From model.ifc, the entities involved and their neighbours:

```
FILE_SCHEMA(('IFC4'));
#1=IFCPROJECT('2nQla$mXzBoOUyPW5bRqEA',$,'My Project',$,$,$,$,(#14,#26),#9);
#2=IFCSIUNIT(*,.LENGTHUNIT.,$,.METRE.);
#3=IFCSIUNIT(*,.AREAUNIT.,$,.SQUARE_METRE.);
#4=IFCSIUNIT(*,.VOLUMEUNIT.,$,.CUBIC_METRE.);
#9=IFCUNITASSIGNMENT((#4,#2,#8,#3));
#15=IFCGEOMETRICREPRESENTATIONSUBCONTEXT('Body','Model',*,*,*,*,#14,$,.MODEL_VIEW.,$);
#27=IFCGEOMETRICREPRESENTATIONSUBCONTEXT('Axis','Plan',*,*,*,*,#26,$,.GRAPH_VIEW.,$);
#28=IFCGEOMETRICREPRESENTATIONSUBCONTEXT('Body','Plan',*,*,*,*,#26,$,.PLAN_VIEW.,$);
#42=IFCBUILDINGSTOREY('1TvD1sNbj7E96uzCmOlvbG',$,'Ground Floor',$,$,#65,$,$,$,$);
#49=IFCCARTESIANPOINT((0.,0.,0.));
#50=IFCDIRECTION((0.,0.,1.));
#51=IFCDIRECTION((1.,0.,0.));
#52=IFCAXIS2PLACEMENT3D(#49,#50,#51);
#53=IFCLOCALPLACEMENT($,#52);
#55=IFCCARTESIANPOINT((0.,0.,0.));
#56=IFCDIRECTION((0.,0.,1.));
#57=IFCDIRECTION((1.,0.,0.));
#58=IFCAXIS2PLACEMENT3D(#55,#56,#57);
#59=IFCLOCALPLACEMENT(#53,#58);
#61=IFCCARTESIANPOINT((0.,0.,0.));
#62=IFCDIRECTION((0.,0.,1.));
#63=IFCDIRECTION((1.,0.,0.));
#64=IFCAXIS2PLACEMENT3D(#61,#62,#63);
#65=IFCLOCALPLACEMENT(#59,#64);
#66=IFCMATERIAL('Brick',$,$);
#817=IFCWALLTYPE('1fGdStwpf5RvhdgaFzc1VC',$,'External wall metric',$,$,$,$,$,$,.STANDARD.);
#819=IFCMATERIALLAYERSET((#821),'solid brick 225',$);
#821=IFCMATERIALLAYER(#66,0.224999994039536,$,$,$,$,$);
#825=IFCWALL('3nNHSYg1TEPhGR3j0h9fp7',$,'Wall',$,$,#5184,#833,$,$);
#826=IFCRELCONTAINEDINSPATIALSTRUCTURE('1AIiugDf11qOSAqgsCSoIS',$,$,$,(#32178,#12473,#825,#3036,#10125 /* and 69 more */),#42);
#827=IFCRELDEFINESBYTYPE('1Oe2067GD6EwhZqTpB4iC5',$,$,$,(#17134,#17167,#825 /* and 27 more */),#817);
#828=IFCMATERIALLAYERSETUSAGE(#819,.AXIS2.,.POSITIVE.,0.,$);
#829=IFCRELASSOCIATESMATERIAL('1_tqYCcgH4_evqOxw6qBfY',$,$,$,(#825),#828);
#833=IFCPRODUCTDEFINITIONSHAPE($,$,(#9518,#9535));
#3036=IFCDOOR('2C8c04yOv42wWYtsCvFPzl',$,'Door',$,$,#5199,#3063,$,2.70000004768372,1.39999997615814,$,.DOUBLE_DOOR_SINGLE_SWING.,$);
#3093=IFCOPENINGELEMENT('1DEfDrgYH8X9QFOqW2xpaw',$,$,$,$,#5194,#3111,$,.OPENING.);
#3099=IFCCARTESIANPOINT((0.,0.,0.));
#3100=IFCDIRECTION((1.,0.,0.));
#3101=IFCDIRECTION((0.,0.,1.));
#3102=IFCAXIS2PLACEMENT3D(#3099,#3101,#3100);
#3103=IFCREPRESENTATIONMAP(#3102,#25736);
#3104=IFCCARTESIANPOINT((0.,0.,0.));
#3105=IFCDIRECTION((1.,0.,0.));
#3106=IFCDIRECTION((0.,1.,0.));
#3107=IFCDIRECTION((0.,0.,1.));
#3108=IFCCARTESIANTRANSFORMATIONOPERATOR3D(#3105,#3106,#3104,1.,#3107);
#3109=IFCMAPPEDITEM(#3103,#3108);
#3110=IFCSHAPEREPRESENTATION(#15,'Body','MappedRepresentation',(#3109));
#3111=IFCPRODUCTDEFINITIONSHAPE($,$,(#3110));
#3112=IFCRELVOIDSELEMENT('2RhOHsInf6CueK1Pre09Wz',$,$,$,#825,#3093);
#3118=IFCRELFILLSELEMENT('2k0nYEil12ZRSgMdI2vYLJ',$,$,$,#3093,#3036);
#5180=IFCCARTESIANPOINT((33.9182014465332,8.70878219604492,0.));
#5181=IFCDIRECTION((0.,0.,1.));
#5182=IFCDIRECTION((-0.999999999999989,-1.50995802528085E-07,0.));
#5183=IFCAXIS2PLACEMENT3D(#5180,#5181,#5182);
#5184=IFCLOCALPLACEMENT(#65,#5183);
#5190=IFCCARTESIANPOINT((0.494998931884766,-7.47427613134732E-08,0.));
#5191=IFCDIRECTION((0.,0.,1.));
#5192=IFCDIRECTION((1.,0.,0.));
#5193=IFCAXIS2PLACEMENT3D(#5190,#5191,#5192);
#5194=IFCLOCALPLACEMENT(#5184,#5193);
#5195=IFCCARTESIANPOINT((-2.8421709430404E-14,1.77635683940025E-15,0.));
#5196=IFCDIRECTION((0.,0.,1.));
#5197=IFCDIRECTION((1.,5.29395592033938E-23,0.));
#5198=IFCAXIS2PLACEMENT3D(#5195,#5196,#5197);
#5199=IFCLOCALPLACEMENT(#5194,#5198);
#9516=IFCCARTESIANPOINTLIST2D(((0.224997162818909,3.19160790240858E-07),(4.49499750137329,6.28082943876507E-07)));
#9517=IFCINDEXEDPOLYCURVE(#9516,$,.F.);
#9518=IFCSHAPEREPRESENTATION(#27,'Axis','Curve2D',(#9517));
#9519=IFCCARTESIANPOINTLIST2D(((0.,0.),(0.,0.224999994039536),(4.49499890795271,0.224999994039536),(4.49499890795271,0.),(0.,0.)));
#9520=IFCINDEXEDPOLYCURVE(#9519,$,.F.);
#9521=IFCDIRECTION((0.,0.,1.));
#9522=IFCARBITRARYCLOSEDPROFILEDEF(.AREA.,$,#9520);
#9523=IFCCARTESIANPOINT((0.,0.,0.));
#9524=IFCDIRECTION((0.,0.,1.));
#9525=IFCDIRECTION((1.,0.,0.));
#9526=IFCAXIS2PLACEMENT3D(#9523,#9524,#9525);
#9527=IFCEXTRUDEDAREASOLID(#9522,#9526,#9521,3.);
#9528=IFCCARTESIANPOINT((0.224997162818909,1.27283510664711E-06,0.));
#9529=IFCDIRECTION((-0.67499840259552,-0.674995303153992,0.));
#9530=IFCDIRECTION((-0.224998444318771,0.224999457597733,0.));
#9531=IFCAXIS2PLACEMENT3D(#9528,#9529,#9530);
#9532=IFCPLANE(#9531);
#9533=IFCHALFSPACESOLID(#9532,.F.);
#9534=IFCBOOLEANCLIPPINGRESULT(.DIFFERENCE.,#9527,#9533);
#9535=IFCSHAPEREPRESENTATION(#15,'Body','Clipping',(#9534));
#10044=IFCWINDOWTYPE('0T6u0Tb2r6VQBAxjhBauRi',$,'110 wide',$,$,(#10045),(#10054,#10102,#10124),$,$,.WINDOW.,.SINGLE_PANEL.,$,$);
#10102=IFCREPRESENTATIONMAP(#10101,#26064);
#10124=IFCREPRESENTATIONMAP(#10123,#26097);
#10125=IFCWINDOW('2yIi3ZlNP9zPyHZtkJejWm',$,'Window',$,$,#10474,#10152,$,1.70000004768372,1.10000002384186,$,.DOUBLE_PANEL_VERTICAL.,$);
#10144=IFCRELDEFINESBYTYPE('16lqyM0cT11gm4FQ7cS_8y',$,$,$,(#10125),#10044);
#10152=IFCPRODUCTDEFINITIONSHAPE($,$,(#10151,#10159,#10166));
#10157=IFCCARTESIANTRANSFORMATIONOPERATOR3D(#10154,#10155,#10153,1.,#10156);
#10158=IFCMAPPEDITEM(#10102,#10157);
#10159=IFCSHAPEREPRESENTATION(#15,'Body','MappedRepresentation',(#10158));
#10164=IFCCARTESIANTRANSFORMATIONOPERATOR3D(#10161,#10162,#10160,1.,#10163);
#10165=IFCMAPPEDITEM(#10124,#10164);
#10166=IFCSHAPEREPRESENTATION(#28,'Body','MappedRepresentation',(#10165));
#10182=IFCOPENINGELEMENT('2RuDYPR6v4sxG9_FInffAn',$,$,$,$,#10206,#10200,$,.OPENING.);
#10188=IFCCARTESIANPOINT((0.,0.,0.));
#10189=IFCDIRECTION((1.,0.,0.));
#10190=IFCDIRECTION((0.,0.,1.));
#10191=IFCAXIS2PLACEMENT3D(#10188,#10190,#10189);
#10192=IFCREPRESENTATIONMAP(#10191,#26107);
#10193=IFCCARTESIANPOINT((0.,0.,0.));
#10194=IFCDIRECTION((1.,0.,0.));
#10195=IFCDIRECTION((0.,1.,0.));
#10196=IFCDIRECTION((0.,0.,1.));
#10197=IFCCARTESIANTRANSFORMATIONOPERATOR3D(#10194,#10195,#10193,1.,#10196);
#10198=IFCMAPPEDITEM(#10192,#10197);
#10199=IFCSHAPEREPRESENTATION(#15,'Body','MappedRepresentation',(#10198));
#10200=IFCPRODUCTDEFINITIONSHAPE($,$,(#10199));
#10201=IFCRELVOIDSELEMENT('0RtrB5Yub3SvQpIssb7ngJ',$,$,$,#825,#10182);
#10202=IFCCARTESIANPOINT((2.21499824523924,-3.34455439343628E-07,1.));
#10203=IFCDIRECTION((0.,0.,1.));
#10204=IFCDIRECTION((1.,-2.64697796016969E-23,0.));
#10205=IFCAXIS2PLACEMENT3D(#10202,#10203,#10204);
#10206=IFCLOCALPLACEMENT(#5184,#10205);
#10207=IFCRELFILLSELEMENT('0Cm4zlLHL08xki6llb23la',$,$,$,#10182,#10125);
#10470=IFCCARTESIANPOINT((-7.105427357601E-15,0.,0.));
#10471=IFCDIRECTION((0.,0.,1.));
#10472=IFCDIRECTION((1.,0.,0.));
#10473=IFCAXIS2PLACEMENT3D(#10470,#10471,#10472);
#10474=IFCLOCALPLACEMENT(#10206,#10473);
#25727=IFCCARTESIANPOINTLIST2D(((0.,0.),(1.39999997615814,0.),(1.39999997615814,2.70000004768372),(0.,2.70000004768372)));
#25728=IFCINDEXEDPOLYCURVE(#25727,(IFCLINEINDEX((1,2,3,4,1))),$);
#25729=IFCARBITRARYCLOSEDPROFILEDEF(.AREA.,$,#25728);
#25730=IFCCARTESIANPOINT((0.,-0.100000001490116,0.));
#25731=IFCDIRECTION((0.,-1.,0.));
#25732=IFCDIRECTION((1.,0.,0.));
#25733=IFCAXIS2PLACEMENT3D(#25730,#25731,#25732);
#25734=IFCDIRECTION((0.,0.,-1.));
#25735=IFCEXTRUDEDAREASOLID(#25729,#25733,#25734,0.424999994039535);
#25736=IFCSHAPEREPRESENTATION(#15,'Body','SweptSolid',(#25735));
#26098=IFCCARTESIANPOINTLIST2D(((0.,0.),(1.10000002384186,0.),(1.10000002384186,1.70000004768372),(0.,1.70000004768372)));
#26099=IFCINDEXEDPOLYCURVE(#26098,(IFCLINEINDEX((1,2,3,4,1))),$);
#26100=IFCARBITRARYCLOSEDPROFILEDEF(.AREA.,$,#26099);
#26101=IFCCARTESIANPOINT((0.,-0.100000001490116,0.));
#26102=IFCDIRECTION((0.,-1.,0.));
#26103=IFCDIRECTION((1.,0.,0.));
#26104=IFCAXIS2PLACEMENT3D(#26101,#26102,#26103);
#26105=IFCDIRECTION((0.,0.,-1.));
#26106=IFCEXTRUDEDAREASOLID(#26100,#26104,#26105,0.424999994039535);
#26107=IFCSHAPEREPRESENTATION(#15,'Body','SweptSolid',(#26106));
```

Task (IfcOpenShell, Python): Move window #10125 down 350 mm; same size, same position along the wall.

```python
import numpy as np
import ifcopenshell
import ifcopenshell.api.geometry
import ifcopenshell.util.placement
import ifcopenshell.util.unit

model = ifcopenshell.open("model.ifc")
unit_scale = ifcopenshell.util.unit.calculate_unit_scale(model)

window = model.by_id(10125)
opening = window.FillsVoids[0].RelatingOpeningElement
dz = -0.35 / unit_scale

shift = np.array([0.0, 0.0, dz])
# The window is placed relative to its opening, so it follows when the opening moves.
matrix = ifcopenshell.util.placement.get_local_placement(opening.ObjectPlacement)
matrix[:3, 3] += shift
ifcopenshell.api.geometry.edit_object_placement(
    model, product=opening, matrix=matrix, is_si=False, should_transform_children=True
)

print(f"moved by {dz * unit_scale:+.3f} m")

model.write("model_edited.ifc")
```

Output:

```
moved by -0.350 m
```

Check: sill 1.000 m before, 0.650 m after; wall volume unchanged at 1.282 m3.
